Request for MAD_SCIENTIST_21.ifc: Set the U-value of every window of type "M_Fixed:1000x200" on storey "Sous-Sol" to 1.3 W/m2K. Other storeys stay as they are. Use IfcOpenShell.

First a look at what the model holds.

```python
import ifcopenshell
import ifcopenshell.util.element

model = ifcopenshell.open("MAD_SCIENTIST_21.ifc")
print(model.schema)
storey = next(s for s in model.by_type("IfcBuildingStorey") if s.Name == "Sous-Sol")
windows = [e for e in ifcopenshell.util.element.get_decomposition(storey) if e.is_a("IfcWindow")]
seen = {}
for e in windows:
    element_type = ifcopenshell.util.element.get_type(e)
    key = (element_type.Name if element_type != e and element_type else None, ifcopenshell.util.element.get_pset(e, "Pset_WindowCommon", "ThermalTransmittance"))
    seen[key] = seen.get(key, 0) + 1
for (name, value), count in sorted(seen.items(), key=str):
    print(count, "x", name, "|", value)
```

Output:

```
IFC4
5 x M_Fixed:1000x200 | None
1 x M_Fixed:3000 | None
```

```python
import ifcopenshell
import ifcopenshell.api.pset
import ifcopenshell.util.element

model = ifcopenshell.open("MAD_SCIENTIST_21.ifc")

storey = next(s for s in model.by_type("IfcBuildingStorey") if s.Name == "Sous-Sol")
windows = [e for e in ifcopenshell.util.element.get_decomposition(storey) if e.is_a("IfcWindow")]

count = 0
for e in windows:
    element_type = ifcopenshell.util.element.get_type(e)
    if element_type in (None, e) or element_type.Name != "M_Fixed:1000x200":
        continue
    # add_pset returns the element's existing set when there is one.
    pset = ifcopenshell.api.pset.add_pset(model, product=e, name="Pset_WindowCommon")
    ifcopenshell.api.pset.edit_pset(model, pset=pset, properties={"ThermalTransmittance": 1.3})
    count += 1

print(count, "windows updated")

model.write("MAD_SCIENTIST_21-out.ifc")
```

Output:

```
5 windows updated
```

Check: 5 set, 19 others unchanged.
